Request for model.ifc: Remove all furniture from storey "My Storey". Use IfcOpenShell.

First a look at what the model holds.

```python
import ifcopenshell
import ifcopenshell.util.element

model = ifcopenshell.open("model.ifc")
print(model.schema)
storey = next(s for s in model.by_type("IfcBuildingStorey") if s.Name == "My Storey")
furniture = [e for e in ifcopenshell.util.element.get_decomposition(storey) if e.is_a("IfcFurnishingElement")]
seen = {}
for e in furniture:
    element_type = ifcopenshell.util.element.get_type(e)
    name = element_type.Name if element_type not in (None, e) else None
    seen[name] = seen.get(name, 0) + 1
for name, count in sorted(seen.items(), key=str):
    print(count, "x", name)
```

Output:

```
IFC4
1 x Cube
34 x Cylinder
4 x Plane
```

```python
import ifcopenshell
import ifcopenshell.api.root
import ifcopenshell.util.element

model = ifcopenshell.open("model.ifc")

storey = next(s for s in model.by_type("IfcBuildingStorey") if s.Name == "My Storey")
furniture = [e for e in ifcopenshell.util.element.get_decomposition(storey) if e.is_a("IfcFurnishingElement")]

for e in furniture:
    ifcopenshell.api.root.remove_product(model, product=e)
print(len(furniture), "removed")

model.write("model_updated.ifc")
```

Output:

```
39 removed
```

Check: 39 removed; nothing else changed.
